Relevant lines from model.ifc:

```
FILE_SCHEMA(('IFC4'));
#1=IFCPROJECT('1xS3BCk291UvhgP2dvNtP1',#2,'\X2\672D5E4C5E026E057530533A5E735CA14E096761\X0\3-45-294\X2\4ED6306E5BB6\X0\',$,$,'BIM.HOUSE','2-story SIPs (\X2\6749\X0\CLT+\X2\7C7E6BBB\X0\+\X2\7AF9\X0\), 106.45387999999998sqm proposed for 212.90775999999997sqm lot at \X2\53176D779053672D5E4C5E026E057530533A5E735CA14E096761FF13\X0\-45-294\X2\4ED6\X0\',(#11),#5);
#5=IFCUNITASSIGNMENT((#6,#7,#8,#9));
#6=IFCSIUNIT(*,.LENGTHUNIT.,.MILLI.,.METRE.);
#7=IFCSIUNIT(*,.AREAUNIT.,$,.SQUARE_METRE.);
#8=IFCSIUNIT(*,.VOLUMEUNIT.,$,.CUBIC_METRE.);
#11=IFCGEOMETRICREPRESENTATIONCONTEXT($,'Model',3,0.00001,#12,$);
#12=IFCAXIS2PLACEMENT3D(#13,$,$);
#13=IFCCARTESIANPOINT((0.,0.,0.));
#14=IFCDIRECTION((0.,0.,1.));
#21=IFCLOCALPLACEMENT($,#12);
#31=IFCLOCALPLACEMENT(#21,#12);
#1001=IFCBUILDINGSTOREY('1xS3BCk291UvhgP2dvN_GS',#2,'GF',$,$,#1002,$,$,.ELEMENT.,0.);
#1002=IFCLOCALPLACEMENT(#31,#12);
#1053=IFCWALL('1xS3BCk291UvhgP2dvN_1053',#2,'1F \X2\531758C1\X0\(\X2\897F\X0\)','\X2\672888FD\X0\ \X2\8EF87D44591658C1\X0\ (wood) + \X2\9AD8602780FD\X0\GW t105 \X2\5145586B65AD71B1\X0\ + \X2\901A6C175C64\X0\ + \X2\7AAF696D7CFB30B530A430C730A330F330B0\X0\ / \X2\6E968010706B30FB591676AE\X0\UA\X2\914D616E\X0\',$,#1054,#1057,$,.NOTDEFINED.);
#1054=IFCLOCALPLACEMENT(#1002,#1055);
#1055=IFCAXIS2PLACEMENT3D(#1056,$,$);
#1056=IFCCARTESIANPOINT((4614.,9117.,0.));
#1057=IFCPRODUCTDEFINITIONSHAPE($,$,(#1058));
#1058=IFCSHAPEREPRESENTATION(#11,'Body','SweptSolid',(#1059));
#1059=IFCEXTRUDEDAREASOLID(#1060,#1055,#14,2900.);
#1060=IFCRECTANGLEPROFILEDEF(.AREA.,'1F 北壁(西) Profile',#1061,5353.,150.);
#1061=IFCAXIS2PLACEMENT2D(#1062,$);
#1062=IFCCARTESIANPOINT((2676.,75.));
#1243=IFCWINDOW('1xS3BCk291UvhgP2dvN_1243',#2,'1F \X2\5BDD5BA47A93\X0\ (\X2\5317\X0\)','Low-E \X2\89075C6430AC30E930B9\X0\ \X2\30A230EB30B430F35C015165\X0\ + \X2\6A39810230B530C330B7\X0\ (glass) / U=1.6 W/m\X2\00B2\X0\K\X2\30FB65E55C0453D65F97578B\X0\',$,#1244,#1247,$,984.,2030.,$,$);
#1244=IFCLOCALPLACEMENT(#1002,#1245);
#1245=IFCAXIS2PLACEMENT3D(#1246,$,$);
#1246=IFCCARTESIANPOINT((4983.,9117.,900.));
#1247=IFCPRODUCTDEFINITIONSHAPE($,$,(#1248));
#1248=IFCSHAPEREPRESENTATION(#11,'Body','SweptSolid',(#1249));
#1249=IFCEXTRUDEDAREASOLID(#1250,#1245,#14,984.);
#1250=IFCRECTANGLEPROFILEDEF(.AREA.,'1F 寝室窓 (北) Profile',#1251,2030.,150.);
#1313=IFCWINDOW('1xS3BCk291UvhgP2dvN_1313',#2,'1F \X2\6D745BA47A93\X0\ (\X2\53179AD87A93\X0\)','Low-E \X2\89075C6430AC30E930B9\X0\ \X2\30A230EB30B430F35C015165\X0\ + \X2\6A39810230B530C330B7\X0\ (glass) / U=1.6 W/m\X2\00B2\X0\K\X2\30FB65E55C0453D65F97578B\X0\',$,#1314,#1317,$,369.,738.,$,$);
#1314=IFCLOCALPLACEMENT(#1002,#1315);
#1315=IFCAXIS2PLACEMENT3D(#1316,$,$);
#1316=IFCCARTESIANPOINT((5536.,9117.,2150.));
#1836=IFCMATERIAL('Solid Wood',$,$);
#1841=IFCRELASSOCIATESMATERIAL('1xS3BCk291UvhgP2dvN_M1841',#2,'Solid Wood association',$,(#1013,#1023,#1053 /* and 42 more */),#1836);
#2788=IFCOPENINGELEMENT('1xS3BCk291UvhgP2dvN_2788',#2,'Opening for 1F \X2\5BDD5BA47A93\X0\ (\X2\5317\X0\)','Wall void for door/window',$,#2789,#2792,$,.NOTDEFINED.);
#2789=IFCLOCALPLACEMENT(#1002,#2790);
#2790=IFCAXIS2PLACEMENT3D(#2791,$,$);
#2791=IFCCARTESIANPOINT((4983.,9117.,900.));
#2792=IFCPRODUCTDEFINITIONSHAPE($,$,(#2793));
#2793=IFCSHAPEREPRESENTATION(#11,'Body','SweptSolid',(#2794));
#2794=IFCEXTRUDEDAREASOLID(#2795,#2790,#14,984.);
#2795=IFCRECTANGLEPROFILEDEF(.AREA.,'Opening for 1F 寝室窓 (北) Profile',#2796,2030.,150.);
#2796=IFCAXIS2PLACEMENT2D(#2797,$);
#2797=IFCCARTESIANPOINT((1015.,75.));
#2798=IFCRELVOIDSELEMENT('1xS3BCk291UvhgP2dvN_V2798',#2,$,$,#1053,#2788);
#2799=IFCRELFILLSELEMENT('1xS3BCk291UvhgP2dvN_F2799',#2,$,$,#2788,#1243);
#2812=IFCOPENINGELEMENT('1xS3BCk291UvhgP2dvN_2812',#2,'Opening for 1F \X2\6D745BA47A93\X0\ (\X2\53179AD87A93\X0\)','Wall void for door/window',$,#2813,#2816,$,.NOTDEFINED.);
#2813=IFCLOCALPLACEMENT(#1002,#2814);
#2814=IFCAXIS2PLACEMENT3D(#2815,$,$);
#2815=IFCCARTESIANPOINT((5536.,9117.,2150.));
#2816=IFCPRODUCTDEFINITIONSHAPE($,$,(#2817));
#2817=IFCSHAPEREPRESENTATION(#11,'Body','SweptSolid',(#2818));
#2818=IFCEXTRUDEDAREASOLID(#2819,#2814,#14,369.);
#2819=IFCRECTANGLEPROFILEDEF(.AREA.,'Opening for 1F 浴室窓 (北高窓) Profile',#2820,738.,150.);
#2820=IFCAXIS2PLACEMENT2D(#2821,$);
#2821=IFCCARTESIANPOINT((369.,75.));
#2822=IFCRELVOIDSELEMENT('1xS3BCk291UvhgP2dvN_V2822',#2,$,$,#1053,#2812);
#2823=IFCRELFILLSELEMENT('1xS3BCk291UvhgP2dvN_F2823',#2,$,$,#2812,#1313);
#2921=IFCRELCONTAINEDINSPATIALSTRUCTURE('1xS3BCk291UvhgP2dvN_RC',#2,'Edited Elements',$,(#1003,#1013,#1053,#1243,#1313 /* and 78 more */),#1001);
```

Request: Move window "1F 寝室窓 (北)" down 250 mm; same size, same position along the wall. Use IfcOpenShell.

```python
import numpy as np
import ifcopenshell
import ifcopenshell.api.geometry
import ifcopenshell.util.placement
import ifcopenshell.util.unit

model = ifcopenshell.open("model.ifc")
unit_scale = ifcopenshell.util.unit.calculate_unit_scale(model)

window = model.by_guid("1xS3BCk291UvhgP2dvN_1243")
opening = window.FillsVoids[0].RelatingOpeningElement
dz = -250.0

shift = np.array([0.0, 0.0, dz])
# The window is not placed relative to its opening, so move both.
for product in (opening, window):
    matrix = ifcopenshell.util.placement.get_local_placement(product.ObjectPlacement)
    matrix[:3, 3] += shift
    ifcopenshell.api.geometry.edit_object_placement(model, product=product, matrix=matrix, is_si=False)

print(f"moved by {dz * unit_scale:+.3f} m")

model.write("model_edited.ifc")
```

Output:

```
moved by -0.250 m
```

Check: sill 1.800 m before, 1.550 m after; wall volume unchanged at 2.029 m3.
